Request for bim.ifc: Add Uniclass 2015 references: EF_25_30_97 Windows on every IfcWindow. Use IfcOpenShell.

First a look at what the model holds.

```python
import ifcopenshell

model = ifcopenshell.open("bim.ifc")
print(model.schema)
print("classifications:", [c.Name for c in model.by_type("IfcClassification")])
for ifc_class in ("IfcDoor", "IfcRoof", "IfcStair", "IfcWall", "IfcWindow"):
    print(ifc_class, len(model.by_type(ifc_class)))
```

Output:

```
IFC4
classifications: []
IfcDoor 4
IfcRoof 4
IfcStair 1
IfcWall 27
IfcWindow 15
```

```python
import ifcopenshell
import ifcopenshell.api.classification

model = ifcopenshell.open("bim.ifc")

system = ifcopenshell.api.classification.add_classification(model, classification="Uniclass 2015")

codes = {
    "IfcWindow": ("EF_25_30_97", "Windows"),
}
for ifc_class, (code, name) in codes.items():
    products = model.by_type(ifc_class)
    ifcopenshell.api.classification.add_reference(
        model, products=products, classification=system, identification=code, name=name
    )
    print(code, len(products))

model.write("bim_v2.ifc")
```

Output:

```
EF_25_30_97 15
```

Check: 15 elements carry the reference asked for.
